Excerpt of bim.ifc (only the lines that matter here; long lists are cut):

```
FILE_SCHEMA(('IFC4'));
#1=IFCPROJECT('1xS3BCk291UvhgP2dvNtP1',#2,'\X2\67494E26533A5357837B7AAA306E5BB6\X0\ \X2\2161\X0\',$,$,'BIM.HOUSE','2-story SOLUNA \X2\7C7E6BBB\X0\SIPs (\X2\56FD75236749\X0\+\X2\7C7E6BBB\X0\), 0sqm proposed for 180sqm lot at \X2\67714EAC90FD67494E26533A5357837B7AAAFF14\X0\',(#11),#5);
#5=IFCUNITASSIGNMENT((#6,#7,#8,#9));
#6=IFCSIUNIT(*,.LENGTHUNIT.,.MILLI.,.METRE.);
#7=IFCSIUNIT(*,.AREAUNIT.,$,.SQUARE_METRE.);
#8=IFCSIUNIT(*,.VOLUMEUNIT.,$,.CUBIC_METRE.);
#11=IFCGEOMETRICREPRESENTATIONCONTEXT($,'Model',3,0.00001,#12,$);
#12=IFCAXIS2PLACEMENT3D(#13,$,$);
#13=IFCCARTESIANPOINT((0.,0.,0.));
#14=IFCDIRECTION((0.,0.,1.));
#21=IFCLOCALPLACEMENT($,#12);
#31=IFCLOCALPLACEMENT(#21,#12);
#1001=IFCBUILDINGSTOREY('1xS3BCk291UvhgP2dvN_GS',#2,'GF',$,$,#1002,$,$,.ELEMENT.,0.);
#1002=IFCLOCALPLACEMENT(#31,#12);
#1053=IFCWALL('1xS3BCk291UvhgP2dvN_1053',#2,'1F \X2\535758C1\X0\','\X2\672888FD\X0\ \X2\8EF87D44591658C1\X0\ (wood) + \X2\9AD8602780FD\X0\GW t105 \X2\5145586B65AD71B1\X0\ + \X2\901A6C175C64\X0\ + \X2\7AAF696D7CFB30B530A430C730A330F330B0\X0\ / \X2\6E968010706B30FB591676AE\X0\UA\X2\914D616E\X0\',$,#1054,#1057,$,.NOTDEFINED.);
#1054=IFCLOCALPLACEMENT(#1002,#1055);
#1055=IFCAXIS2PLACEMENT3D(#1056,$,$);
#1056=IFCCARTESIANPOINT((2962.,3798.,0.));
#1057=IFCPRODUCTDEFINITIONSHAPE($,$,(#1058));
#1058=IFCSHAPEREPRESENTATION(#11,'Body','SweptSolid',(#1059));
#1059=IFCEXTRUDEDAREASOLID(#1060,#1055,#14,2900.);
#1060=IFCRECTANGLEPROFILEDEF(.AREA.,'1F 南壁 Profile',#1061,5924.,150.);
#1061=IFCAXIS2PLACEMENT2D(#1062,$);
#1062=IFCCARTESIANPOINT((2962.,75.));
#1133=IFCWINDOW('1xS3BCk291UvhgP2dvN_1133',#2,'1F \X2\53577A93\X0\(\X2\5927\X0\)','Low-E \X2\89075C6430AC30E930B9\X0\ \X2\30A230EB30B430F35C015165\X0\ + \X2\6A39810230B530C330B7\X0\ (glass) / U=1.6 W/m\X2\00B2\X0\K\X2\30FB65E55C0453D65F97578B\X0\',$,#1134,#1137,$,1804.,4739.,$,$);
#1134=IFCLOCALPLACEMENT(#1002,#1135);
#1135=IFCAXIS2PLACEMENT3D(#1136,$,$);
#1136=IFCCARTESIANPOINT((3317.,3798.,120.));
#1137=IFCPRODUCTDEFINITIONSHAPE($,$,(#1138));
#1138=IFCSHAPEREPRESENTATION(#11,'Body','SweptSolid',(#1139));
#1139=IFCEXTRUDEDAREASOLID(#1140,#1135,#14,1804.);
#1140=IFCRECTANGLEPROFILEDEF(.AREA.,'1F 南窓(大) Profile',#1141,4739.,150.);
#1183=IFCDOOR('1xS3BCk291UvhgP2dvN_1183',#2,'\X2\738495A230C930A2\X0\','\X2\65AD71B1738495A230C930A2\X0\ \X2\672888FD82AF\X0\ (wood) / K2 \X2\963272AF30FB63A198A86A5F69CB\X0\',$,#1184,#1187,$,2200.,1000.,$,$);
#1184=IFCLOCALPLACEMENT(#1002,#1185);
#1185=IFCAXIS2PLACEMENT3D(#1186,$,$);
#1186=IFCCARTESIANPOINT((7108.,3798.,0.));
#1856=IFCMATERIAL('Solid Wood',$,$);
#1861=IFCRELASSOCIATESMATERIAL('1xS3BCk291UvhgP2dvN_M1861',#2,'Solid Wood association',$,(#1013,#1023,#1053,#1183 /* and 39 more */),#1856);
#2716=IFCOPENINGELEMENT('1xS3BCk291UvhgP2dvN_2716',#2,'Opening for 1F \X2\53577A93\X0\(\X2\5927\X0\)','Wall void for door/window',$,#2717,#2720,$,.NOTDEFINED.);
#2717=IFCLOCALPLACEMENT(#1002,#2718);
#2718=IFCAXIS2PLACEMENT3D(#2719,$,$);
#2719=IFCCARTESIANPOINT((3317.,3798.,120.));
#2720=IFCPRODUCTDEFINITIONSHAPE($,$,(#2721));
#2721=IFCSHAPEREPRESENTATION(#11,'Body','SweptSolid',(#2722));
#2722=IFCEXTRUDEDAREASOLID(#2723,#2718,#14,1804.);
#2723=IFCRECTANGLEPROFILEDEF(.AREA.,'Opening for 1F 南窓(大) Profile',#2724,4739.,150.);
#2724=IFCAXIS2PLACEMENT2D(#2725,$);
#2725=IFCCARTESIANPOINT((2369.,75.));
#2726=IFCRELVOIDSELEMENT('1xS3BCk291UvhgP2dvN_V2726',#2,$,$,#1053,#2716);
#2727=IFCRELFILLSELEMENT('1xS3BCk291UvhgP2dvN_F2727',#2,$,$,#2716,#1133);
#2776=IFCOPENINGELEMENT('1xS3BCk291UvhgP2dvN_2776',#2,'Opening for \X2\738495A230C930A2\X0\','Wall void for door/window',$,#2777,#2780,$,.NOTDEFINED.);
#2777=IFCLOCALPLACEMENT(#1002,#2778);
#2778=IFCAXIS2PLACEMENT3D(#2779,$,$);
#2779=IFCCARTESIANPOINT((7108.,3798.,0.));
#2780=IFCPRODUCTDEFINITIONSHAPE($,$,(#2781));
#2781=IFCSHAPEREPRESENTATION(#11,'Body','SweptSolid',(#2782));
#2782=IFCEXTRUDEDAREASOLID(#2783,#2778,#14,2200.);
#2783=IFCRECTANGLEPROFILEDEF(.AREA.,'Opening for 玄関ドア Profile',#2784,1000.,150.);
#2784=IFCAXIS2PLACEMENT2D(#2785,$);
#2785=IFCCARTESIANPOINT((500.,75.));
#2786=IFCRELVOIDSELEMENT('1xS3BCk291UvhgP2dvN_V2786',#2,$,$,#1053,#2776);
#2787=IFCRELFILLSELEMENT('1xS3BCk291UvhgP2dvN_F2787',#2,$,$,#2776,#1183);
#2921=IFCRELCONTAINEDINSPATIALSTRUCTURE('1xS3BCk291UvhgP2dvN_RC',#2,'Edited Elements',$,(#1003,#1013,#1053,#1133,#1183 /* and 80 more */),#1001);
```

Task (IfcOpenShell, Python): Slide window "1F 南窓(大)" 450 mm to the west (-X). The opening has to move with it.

```python
import ifcopenshell
import ifcopenshell.api.geometry
import ifcopenshell.util.placement
import ifcopenshell.util.unit

model = ifcopenshell.open("bim.ifc")
unit_scale = ifcopenshell.util.unit.calculate_unit_scale(model)

window = model.by_id(1133)
opening = window.FillsVoids[0].RelatingOpeningElement
wall = opening.VoidsElements[0].RelatingBuildingElement

wall_matrix = ifcopenshell.util.placement.get_local_placement(wall.ObjectPlacement)
shift = wall_matrix[:3, 0] * -0.45 / unit_scale
before = ifcopenshell.util.placement.get_local_placement(window.ObjectPlacement)[:3, 3].copy()

# The window is not placed relative to its opening, so move both.
for product in (opening, window):
    matrix = ifcopenshell.util.placement.get_local_placement(product.ObjectPlacement)
    matrix[:3, 3] += shift
    ifcopenshell.api.geometry.edit_object_placement(model, product=product, matrix=matrix, is_si=False)

after = ifcopenshell.util.placement.get_local_placement(window.ObjectPlacement)[:3, 3]
print("window moved by", (after - before).round(3) + 0.0)

model.write("bim_updated.ifc")
```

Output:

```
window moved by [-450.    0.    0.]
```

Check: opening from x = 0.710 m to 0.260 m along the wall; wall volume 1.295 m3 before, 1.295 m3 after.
